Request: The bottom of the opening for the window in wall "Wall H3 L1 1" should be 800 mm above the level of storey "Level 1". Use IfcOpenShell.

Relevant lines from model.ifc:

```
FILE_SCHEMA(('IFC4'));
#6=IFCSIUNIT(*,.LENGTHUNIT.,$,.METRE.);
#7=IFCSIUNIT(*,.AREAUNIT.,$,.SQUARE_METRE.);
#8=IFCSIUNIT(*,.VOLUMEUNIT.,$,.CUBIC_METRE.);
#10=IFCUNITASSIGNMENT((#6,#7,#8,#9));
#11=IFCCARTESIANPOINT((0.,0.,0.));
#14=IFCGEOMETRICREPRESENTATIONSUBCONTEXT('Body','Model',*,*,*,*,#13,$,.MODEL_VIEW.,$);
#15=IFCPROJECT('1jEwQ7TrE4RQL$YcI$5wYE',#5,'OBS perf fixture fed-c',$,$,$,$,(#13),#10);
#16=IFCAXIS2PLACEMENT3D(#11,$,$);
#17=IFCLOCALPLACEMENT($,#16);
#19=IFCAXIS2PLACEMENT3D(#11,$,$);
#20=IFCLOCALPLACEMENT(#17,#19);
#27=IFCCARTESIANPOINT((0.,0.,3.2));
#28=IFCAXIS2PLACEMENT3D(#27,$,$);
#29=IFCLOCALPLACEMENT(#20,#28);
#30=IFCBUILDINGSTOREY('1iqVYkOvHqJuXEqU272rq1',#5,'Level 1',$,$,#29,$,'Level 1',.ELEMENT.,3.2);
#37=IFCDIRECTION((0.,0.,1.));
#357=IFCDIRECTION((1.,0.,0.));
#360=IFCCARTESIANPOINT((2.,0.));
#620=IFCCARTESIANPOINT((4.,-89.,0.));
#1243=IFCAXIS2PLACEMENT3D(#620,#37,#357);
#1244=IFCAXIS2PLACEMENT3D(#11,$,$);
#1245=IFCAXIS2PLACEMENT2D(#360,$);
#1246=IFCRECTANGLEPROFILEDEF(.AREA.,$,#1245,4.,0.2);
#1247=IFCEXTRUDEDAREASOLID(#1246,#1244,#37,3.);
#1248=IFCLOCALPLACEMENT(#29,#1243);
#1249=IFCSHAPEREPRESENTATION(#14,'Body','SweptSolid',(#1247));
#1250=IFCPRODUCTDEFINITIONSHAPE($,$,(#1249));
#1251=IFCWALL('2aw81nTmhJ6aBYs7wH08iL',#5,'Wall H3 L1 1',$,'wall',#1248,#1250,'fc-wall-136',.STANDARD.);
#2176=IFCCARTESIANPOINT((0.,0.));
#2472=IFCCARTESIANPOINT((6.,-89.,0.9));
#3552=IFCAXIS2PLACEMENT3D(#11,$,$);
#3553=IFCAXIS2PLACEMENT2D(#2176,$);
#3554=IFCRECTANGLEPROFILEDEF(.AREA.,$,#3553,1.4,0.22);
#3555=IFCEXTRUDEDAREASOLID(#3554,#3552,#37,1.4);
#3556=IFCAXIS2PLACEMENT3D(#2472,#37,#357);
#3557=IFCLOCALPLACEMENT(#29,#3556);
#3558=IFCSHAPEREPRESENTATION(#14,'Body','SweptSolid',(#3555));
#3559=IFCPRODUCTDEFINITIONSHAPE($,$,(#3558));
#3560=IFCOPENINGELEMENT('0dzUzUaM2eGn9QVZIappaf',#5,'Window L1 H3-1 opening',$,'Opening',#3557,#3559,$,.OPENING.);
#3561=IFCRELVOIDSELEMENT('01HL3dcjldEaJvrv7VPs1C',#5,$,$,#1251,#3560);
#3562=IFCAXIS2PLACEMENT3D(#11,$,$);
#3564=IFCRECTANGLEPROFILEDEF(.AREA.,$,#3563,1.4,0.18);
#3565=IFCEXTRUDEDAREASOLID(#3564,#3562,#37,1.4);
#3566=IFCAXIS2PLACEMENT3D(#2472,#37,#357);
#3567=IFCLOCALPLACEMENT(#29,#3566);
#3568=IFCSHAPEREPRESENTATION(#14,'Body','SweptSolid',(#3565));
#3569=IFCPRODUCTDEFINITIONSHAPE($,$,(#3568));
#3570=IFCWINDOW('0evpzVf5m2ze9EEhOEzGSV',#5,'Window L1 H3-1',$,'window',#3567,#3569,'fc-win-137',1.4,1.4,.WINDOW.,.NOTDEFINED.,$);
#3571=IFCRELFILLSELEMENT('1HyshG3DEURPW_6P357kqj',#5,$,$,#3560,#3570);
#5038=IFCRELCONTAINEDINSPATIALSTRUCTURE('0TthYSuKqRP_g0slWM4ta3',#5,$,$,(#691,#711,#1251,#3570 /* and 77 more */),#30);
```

```python
import numpy as np
import ifcopenshell
import ifcopenshell.api.geometry
import ifcopenshell.geom
import ifcopenshell.util.element
import ifcopenshell.util.placement
import ifcopenshell.util.shape
import ifcopenshell.util.unit

model = ifcopenshell.open("model.ifc")
unit_scale = ifcopenshell.util.unit.calculate_unit_scale(model)

window = model.by_id(3570)
opening = window.FillsVoids[0].RelatingOpeningElement
storey = ifcopenshell.util.element.get_container(window, ifc_class="IfcBuildingStorey")
level = ifcopenshell.util.placement.get_local_placement(storey.ObjectPlacement)[2, 3]

# The opening's origin need not be at the sill, so measure its lowest point.
shape = ifcopenshell.geom.create_shape(ifcopenshell.geom.settings(), opening)
bottom = ifcopenshell.util.shape.get_shape_bottom_elevation(shape, shape.geometry) / unit_scale
dz = level + 0.8 / unit_scale - bottom

shift = np.array([0.0, 0.0, dz])
# The window is not placed relative to its opening, so move both.
for product in (opening, window):
    matrix = ifcopenshell.util.placement.get_local_placement(product.ObjectPlacement)
    matrix[:3, 3] += shift
    ifcopenshell.api.geometry.edit_object_placement(model, product=product, matrix=matrix, is_si=False)

print(f"moved by {dz * unit_scale:+.3f} m")

model.write("model_v2.ifc")
```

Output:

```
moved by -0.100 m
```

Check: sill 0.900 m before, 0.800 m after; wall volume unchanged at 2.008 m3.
